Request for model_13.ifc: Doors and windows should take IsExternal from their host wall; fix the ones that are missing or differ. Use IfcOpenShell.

First a look at what the model holds.

```python
import ifcopenshell
import ifcopenshell.util.element

model = ifcopenshell.open("model_13.ifc")
print(model.schema)
seen = {}
for e in model.by_type("IfcDoor") + model.by_type("IfcWindow"):
    if not e.FillsVoids:
        continue
    host = e.FillsVoids[0].RelatingOpeningElement.VoidsElements[0].RelatingBuildingElement
    own = ifcopenshell.util.element.get_pset(e, f"Pset_{e.is_a()[3:].removesuffix('StandardCase')}Common", "IsExternal")
    wall = ifcopenshell.util.element.get_pset(host, "Pset_WallCommon", "IsExternal")
    seen[e.is_a(), own, wall] = seen.get((e.is_a(), own, wall), 0) + 1
for (cls, own, wall), count in sorted(seen.items(), key=str):
    print(count, cls, "IsExternal:", own, "| host wall:", wall)
```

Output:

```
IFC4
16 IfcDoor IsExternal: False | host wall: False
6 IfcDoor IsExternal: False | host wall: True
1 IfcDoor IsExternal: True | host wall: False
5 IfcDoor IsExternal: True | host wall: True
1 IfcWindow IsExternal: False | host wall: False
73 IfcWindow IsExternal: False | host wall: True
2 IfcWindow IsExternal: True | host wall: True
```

```python
import ifcopenshell
import ifcopenshell.api.pset
import ifcopenshell.util.element

model = ifcopenshell.open("model_13.ifc")

count = 0
for ifc_class, pset_name in (("IfcDoor", "Pset_DoorCommon"), ("IfcWindow", "Pset_WindowCommon")):
    for e in model.by_type(ifc_class):
        if not e.FillsVoids:
            continue
        host = e.FillsVoids[0].RelatingOpeningElement.VoidsElements[0].RelatingBuildingElement
        external = ifcopenshell.util.element.get_pset(host, "Pset_WallCommon", "IsExternal")
        if external is None or ifcopenshell.util.element.get_pset(e, pset_name, "IsExternal") == external:
            continue
        pset = ifcopenshell.api.pset.add_pset(model, product=e, name=pset_name)
        ifcopenshell.api.pset.edit_pset(model, pset=pset, properties={"IsExternal": external})
        count += 1

print(count, "updated")

model.write("model_13_v2.ifc")
```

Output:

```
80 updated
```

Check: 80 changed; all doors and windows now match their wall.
